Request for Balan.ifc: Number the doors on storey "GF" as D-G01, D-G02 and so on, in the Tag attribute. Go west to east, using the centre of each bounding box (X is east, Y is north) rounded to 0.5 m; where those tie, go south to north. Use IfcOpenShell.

First a look at what the model holds.

```python
import ifcopenshell
import ifcopenshell.util.element
import ifcopenshell.util.placement

model = ifcopenshell.open("Balan.ifc")
print(model.schema)
storey = next(s for s in model.by_type("IfcBuildingStorey") if s.Name == "GF")
doors = [e for e in ifcopenshell.util.element.get_decomposition(storey) if e.is_a("IfcDoor")]
for e in sorted(doors, key=lambda e: e.id()):
    origin = ifcopenshell.util.placement.get_local_placement(e.ObjectPlacement)[:3, 3]
    print(e.id(), e.Tag, e.Name, origin.round(2) + 0.0, sep=" | ")
```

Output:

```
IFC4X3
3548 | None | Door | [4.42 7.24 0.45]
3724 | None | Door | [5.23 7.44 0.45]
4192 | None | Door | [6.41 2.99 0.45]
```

```python
import ifcopenshell
import ifcopenshell.geom
import ifcopenshell.util.element
import ifcopenshell.util.shape

model = ifcopenshell.open("Balan.ifc")
settings = ifcopenshell.geom.settings()
settings.set("use-world-coords", True)


def centre(element):
    shape = ifcopenshell.geom.create_shape(settings, element)
    return ifcopenshell.util.shape.get_bbox_centroid(shape.geometry)


storey = next(s for s in model.by_type("IfcBuildingStorey") if s.Name == "GF")
doors = [e for e in ifcopenshell.util.element.get_decomposition(storey) if e.is_a("IfcDoor")]

# Insertion points can sit at a corner or the storey origin, so sort by the geometry (in metres).
centres = {e: centre(e) for e in doors}
doors.sort(key=lambda e: (round(centres[e][0] / 0.5), centres[e][1]))

for i, e in enumerate(doors, start=1):
    number = f"D-G{i:02d}"
    e.Tag = number
    print(e.id(), number)

model.write("Balan-out.ifc")
```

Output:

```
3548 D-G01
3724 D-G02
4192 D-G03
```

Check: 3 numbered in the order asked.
